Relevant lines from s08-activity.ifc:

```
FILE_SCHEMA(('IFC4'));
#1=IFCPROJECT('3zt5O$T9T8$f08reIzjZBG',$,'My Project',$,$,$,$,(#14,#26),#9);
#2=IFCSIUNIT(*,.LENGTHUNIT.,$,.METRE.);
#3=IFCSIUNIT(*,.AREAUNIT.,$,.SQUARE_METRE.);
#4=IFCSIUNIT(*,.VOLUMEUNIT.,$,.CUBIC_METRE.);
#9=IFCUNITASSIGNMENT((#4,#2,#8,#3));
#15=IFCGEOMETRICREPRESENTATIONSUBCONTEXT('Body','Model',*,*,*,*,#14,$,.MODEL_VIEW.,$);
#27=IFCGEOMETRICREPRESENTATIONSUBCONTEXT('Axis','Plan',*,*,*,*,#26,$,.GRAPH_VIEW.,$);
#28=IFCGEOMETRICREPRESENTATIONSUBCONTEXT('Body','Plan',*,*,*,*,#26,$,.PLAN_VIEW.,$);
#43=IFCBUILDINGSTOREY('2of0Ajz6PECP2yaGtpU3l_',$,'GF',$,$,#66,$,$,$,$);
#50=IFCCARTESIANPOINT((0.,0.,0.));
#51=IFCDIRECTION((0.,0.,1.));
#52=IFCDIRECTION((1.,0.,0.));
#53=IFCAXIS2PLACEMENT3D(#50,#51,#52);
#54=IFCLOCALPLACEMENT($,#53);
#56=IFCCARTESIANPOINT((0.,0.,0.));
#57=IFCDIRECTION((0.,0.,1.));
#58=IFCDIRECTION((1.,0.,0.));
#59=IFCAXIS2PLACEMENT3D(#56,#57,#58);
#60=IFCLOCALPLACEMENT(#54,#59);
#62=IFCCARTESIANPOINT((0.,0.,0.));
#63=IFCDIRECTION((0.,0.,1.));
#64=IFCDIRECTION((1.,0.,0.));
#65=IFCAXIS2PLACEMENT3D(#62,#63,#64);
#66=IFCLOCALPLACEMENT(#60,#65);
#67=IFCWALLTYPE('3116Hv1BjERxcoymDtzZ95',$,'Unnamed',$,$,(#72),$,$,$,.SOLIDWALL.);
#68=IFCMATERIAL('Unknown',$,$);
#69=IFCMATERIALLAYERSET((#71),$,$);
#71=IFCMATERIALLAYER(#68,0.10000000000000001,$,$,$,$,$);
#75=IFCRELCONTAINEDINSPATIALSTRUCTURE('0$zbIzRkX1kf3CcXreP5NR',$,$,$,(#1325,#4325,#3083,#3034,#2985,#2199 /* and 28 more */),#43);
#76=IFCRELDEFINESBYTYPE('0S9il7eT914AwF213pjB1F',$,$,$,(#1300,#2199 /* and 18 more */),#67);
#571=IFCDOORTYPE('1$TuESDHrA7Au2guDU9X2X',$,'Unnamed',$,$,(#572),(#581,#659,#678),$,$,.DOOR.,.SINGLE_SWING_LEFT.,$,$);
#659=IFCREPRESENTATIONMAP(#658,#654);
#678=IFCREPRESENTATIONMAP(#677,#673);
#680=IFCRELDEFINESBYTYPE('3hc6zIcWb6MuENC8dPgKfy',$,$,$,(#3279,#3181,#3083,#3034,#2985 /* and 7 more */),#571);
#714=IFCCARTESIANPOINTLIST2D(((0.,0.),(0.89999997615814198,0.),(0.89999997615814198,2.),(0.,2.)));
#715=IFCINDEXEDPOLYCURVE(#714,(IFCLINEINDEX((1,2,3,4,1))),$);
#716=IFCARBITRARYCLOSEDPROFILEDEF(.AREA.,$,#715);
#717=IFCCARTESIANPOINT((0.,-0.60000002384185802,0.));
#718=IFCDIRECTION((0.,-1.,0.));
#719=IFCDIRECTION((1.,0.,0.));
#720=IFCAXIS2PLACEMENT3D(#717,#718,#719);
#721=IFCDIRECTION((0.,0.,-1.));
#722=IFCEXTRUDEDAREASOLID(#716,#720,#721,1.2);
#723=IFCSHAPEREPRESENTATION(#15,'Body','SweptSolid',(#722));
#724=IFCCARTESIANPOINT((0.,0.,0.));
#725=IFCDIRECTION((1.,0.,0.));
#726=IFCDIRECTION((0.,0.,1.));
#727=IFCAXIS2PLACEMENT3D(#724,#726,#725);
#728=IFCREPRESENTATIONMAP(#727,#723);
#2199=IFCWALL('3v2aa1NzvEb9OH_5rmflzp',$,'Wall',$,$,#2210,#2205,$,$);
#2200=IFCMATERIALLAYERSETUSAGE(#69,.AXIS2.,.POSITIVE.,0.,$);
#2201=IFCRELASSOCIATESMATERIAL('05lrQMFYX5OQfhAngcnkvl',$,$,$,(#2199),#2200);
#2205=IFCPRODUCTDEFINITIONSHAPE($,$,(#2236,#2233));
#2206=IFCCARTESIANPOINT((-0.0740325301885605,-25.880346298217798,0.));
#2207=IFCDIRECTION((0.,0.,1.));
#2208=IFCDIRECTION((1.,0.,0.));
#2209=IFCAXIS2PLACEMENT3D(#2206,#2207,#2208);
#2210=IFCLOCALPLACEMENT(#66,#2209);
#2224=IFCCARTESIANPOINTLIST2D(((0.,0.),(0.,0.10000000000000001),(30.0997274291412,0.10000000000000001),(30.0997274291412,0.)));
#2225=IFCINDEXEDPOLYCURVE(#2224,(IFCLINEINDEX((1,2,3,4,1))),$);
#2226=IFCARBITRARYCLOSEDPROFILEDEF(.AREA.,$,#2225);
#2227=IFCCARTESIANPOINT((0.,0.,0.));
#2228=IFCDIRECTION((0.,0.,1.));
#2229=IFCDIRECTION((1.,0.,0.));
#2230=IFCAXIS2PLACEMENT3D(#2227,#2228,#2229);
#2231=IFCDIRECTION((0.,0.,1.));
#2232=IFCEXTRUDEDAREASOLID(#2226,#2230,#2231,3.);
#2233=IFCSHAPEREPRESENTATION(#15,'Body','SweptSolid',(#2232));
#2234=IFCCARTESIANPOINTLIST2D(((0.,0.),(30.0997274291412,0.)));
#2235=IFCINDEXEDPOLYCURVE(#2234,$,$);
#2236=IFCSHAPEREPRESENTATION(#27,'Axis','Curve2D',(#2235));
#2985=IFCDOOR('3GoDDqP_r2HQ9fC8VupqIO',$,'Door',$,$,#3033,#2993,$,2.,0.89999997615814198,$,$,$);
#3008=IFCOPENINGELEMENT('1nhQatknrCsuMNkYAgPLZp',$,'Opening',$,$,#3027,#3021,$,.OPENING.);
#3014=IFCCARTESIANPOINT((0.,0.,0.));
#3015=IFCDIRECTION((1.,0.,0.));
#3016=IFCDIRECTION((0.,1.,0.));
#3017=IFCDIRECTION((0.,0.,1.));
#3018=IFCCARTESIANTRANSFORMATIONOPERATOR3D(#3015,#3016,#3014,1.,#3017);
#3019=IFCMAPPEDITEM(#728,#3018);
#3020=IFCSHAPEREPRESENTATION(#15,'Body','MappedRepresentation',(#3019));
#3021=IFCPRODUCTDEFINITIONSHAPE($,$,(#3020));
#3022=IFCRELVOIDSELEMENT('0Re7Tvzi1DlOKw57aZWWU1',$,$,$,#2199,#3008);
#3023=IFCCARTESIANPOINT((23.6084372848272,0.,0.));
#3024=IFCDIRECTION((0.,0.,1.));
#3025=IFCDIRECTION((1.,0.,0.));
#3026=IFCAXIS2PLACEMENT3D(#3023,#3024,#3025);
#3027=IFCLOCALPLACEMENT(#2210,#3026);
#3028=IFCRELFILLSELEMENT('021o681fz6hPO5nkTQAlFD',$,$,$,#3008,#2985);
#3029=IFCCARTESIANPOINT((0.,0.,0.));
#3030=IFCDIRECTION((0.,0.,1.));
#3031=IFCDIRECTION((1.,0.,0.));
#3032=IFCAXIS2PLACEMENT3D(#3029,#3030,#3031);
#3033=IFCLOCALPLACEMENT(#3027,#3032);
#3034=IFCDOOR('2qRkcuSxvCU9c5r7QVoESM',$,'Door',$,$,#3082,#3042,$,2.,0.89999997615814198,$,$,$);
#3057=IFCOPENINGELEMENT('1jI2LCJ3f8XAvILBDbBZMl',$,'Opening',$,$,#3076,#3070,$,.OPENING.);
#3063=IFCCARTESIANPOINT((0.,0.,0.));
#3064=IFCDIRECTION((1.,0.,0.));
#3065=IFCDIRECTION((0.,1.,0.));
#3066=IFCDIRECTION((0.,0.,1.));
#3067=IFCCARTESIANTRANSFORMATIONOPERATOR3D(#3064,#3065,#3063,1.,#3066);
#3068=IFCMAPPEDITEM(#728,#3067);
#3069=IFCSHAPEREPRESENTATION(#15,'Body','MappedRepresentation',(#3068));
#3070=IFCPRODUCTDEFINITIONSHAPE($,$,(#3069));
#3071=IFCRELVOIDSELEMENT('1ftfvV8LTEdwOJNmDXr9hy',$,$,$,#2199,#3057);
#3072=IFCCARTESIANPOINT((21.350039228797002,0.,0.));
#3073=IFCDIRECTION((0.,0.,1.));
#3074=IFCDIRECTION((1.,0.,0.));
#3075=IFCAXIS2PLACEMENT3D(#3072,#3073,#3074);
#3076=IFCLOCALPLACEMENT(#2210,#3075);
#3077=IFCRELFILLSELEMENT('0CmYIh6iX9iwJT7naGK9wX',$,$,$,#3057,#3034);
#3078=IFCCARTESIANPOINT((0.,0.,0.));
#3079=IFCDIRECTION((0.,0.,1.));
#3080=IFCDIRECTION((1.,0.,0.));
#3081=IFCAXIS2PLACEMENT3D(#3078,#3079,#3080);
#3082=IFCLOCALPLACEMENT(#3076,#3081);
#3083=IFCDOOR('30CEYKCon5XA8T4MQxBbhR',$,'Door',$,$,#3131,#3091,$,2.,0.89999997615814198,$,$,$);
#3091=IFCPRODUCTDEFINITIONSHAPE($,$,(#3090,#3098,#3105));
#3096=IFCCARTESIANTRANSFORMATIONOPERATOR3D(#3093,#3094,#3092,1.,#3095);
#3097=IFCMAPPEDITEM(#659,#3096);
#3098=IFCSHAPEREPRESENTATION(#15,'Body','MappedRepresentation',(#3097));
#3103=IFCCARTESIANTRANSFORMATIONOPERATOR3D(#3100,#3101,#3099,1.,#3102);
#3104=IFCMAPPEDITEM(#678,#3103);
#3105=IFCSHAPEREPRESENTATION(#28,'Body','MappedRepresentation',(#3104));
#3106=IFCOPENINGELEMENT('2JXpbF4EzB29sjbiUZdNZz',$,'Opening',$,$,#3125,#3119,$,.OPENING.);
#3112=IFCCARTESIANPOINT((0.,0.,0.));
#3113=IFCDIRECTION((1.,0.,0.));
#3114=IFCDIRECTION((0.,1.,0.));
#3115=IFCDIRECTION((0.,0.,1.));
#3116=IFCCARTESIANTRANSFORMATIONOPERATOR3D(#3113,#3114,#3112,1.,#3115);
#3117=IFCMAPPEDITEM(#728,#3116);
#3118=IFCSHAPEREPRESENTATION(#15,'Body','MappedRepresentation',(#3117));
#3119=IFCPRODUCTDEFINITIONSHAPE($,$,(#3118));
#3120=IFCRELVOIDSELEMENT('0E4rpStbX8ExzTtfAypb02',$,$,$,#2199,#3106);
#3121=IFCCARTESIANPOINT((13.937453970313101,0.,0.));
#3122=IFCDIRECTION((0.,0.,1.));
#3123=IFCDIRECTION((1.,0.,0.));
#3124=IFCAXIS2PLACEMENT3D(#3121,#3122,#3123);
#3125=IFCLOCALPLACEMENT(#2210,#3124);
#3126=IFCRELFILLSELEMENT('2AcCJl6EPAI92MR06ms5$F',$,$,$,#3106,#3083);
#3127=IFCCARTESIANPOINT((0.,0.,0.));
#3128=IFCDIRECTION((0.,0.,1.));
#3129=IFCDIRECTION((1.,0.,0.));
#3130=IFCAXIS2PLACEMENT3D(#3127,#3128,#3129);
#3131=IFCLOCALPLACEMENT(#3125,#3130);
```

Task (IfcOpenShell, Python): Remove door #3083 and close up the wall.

```python
import ifcopenshell
import ifcopenshell.api.feature
import ifcopenshell.api.root
import ifcopenshell.geom
import ifcopenshell.util.shape

model = ifcopenshell.open("s08-activity.ifc")
settings = ifcopenshell.geom.settings()


def volume(element):
    """Net volume in cubic metres, openings subtracted."""
    shape = ifcopenshell.geom.create_shape(settings, element)
    return ifcopenshell.util.shape.get_volume(shape.geometry)


door = model.by_guid("30CEYKCon5XA8T4MQxBbhR")
opening = door.FillsVoids[0].RelatingOpeningElement
wall = opening.VoidsElements[0].RelatingBuildingElement
before = volume(wall)

ifcopenshell.api.root.remove_product(model, product=door)
ifcopenshell.api.feature.remove_feature(model, feature=opening)

after = volume(wall)

print(f"wall volume {before:.3f} -> {after:.3f} m3")

model.write("s08-activity-out.ifc")
```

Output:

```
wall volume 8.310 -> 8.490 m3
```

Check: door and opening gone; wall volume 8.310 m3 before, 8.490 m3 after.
